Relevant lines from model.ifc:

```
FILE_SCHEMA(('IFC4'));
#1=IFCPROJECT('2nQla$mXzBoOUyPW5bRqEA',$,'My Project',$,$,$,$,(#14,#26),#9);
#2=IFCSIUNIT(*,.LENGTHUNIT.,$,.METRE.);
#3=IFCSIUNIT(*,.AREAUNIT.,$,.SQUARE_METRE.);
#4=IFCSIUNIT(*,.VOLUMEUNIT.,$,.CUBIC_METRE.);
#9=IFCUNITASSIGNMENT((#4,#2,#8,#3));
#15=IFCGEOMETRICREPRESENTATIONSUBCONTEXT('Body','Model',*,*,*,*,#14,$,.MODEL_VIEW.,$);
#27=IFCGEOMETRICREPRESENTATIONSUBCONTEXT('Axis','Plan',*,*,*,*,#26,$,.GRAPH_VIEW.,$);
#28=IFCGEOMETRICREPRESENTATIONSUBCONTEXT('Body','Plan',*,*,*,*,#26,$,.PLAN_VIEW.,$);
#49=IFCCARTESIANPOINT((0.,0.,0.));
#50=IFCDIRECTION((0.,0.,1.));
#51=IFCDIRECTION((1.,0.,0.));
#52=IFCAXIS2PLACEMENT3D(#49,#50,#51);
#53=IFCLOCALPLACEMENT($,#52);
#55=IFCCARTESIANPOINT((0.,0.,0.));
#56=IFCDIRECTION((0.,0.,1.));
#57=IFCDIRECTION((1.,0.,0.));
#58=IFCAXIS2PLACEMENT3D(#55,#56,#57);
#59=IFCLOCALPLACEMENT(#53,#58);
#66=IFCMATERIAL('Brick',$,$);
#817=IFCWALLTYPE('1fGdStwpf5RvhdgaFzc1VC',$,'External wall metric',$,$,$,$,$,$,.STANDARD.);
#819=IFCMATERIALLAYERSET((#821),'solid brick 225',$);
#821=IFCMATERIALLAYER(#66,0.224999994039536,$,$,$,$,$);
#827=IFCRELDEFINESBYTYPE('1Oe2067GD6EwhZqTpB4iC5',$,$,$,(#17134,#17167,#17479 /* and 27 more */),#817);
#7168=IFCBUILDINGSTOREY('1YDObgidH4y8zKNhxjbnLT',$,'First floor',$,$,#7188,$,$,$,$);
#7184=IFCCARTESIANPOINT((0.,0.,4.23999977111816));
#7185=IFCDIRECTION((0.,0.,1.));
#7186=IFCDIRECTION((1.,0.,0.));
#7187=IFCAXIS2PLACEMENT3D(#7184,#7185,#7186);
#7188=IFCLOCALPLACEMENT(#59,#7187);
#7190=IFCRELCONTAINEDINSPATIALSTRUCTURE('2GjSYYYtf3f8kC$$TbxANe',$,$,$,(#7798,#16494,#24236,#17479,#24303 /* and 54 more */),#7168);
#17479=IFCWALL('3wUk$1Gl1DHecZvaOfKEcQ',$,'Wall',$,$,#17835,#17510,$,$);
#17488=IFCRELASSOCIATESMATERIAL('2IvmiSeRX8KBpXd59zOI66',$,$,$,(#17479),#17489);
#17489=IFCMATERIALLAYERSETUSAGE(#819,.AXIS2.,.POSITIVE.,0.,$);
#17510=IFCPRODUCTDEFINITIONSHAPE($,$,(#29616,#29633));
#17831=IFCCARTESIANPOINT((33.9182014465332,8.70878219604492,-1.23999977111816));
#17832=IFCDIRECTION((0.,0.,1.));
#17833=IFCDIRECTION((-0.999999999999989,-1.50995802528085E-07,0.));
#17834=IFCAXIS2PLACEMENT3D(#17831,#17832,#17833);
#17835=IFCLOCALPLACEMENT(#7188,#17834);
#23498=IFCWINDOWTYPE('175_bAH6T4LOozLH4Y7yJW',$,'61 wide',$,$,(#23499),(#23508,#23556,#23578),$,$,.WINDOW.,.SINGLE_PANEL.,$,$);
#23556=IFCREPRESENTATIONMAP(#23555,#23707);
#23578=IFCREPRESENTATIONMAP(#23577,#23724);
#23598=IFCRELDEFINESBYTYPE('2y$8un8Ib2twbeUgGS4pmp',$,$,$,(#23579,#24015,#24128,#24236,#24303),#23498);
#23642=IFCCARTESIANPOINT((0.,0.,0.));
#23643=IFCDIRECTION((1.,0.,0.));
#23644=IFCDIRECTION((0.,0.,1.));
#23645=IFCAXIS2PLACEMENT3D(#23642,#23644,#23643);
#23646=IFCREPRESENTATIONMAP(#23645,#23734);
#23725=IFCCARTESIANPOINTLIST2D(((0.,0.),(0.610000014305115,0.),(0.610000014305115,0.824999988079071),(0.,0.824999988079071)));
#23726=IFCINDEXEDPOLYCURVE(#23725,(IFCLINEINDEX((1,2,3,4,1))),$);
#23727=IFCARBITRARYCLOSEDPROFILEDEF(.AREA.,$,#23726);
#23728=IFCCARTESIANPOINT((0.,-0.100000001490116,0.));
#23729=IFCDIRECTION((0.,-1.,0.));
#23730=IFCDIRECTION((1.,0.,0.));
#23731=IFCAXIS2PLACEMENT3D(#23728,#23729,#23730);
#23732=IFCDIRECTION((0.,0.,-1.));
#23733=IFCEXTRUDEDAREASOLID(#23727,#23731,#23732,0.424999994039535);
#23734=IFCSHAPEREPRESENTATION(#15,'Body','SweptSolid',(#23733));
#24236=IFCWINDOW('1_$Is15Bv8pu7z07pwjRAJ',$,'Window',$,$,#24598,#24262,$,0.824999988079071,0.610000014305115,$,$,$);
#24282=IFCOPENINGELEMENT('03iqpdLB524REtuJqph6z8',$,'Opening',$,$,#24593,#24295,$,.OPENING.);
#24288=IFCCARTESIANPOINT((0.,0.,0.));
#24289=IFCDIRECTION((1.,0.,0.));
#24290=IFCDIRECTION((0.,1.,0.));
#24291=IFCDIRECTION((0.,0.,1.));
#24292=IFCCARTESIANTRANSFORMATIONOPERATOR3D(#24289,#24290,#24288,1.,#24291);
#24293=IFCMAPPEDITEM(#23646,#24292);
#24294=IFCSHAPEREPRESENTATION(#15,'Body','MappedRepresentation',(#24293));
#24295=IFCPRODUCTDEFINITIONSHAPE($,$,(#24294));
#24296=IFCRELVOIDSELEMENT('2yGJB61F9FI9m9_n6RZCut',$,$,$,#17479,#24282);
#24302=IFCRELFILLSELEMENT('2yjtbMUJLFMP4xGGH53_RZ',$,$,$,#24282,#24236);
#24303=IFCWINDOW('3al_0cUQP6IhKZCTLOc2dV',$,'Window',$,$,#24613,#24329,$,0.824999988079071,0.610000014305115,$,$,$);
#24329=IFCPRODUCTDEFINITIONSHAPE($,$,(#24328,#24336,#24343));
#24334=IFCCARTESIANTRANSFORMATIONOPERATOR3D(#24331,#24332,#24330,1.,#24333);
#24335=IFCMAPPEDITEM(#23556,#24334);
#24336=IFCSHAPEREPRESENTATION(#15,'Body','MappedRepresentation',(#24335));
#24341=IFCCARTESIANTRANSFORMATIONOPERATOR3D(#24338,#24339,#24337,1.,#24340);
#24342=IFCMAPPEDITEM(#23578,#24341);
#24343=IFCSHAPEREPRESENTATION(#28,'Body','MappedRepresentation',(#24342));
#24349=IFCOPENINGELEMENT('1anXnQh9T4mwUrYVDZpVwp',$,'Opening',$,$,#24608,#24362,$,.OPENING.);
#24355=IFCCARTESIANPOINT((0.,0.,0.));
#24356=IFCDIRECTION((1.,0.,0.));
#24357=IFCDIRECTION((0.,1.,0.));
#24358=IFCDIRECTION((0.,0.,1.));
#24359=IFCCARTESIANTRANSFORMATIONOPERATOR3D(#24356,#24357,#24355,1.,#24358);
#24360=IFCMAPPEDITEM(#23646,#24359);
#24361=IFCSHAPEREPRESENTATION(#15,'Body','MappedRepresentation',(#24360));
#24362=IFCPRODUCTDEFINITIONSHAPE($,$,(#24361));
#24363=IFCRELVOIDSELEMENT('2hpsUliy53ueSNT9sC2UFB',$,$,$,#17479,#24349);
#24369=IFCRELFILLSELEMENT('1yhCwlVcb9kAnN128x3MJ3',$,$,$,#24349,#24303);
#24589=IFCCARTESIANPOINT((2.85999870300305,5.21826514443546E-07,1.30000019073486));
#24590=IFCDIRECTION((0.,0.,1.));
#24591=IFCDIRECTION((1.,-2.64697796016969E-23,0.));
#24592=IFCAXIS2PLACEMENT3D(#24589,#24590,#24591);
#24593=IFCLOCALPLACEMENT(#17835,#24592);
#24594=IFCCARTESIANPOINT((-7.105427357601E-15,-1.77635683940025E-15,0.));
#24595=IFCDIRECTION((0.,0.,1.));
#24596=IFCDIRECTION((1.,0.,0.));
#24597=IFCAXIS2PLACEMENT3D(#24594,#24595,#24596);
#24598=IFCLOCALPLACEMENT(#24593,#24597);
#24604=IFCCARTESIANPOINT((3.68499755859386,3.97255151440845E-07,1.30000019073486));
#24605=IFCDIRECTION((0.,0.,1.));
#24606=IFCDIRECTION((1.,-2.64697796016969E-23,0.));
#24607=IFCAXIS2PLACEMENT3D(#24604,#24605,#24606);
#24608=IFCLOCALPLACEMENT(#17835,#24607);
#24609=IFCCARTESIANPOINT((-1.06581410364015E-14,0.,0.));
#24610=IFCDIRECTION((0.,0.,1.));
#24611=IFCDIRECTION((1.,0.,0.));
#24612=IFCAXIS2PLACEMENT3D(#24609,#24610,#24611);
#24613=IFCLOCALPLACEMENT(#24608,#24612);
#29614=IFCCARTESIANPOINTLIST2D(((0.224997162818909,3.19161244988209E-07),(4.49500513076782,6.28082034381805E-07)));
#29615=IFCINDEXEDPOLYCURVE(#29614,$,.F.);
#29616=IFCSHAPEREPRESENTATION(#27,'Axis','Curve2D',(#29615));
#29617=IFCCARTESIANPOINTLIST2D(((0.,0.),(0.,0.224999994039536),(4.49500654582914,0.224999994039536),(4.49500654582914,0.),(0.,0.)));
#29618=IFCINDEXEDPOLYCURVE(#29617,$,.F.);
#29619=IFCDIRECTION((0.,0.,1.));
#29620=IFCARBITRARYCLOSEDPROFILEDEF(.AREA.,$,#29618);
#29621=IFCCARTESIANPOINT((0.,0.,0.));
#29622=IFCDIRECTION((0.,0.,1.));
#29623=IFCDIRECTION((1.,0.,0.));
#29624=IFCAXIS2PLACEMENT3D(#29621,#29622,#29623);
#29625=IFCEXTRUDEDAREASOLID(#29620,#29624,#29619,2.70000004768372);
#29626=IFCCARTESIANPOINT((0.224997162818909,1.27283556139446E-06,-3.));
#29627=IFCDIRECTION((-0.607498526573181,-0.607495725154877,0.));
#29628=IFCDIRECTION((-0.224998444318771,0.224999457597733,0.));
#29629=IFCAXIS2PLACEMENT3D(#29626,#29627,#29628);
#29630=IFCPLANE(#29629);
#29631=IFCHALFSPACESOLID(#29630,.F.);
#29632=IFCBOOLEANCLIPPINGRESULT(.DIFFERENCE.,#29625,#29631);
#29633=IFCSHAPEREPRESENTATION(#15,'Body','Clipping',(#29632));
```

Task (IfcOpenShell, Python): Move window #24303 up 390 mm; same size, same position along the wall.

```python
import numpy as np
import ifcopenshell
import ifcopenshell.api.geometry
import ifcopenshell.util.placement
import ifcopenshell.util.unit

model = ifcopenshell.open("model.ifc")
unit_scale = ifcopenshell.util.unit.calculate_unit_scale(model)

window = model.by_guid("3al_0cUQP6IhKZCTLOc2dV")
opening = window.FillsVoids[0].RelatingOpeningElement
dz = 0.39

shift = np.array([0.0, 0.0, dz])
# The window is placed relative to its opening, so it follows when the opening moves.
matrix = ifcopenshell.util.placement.get_local_placement(opening.ObjectPlacement)
matrix[:3, 3] += shift
ifcopenshell.api.geometry.edit_object_placement(
    model, product=opening, matrix=matrix, is_si=False, should_transform_children=True
)

print(f"moved by {dz * unit_scale:+.3f} m")

model.write("model_edited.ifc")
```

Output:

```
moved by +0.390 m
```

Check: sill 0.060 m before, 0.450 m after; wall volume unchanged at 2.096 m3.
